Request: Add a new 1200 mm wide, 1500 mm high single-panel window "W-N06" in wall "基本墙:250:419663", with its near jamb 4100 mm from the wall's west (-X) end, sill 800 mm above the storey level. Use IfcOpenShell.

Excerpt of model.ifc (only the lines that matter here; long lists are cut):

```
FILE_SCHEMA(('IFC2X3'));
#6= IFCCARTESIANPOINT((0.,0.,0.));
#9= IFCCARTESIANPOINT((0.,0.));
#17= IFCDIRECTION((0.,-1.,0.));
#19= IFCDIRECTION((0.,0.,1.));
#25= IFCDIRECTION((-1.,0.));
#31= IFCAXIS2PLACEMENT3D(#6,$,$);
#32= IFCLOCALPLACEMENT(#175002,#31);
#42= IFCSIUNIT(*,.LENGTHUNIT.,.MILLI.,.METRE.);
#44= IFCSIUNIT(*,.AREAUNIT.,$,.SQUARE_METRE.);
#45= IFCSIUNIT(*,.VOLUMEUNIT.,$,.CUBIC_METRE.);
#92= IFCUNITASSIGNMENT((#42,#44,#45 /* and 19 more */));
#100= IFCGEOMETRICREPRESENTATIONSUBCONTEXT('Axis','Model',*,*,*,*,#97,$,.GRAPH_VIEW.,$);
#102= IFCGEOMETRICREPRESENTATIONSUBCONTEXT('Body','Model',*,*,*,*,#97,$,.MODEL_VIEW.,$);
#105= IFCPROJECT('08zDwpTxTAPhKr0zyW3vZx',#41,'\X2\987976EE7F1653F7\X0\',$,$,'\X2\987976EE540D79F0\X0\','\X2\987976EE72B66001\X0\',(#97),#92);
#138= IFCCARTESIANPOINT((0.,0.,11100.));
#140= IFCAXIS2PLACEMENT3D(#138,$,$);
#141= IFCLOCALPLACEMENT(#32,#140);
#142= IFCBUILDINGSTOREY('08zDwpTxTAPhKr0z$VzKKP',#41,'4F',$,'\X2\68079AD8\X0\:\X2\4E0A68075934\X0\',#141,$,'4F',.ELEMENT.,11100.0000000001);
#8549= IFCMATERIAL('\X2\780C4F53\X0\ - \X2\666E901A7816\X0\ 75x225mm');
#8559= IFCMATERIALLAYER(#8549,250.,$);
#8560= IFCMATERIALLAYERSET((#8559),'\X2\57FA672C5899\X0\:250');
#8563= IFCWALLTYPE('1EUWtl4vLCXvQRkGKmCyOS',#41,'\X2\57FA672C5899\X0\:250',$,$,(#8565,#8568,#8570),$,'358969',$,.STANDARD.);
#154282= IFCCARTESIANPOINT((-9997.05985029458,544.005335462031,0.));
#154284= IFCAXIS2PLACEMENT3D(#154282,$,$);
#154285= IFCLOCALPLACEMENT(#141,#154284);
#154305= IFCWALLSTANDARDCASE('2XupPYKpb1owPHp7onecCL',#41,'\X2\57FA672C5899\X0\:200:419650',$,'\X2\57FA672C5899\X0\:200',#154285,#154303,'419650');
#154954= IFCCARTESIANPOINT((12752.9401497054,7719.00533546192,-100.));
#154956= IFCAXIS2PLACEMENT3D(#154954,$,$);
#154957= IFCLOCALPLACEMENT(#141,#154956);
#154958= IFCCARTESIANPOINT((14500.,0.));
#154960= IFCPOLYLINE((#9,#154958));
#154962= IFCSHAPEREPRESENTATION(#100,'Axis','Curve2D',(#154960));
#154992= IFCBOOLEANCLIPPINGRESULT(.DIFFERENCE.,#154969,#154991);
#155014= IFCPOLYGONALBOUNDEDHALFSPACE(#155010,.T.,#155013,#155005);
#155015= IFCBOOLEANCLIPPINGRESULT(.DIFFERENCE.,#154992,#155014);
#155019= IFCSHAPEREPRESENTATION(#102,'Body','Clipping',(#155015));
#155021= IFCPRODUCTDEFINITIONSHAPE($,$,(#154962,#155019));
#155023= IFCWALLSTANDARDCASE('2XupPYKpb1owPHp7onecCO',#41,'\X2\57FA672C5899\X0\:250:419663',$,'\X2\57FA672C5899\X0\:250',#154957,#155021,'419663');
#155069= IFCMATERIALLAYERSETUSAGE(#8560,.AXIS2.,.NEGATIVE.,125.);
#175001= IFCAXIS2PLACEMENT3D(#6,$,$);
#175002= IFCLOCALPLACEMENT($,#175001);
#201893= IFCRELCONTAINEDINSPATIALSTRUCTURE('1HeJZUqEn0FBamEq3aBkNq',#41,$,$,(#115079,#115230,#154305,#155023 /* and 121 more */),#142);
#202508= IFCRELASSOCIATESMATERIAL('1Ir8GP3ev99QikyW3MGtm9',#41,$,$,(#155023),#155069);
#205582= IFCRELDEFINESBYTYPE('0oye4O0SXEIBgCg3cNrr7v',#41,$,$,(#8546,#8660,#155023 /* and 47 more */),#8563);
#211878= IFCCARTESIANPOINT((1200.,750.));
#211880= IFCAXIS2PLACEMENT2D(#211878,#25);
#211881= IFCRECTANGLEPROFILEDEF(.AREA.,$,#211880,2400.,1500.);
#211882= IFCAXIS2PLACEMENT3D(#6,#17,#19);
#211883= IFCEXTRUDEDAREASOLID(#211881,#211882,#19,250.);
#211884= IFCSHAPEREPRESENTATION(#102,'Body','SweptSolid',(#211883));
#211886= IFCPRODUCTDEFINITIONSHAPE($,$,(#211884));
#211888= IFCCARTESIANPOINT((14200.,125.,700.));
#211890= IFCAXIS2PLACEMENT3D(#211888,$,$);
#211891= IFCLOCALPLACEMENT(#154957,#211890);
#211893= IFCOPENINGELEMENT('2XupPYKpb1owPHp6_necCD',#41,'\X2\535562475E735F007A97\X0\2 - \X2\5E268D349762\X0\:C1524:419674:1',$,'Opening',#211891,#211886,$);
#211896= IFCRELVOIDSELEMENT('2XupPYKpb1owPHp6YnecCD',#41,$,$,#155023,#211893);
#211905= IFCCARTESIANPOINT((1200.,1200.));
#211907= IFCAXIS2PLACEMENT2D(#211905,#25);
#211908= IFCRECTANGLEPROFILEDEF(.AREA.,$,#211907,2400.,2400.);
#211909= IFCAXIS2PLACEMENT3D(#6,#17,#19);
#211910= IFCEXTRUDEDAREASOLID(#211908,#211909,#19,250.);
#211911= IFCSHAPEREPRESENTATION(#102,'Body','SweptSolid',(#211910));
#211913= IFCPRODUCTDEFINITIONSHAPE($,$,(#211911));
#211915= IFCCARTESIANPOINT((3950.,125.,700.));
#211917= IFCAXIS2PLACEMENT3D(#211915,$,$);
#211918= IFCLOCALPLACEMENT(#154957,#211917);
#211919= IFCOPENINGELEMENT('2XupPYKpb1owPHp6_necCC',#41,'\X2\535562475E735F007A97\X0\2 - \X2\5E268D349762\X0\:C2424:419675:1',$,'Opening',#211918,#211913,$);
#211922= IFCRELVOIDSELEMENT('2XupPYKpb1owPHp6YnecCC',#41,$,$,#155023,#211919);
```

```python
import numpy as np
import ifcopenshell
import ifcopenshell.api.feature
import ifcopenshell.api.geometry
import ifcopenshell.api.root
import ifcopenshell.api.spatial
import ifcopenshell.api.type
import ifcopenshell.geom
import ifcopenshell.util.element
import ifcopenshell.util.placement
import ifcopenshell.util.representation
import ifcopenshell.util.shape
import ifcopenshell.util.unit

model = ifcopenshell.open("model.ifc")
unit_scale = ifcopenshell.util.unit.calculate_unit_scale(model)
settings = ifcopenshell.geom.settings()


def volume(element):
    """Net volume in cubic metres, openings subtracted."""
    shape = ifcopenshell.geom.create_shape(settings, element)
    return ifcopenshell.util.shape.get_volume(shape.geometry)


wall = model.by_guid("2XupPYKpb1owPHp7onecCO")
storey = ifcopenshell.util.element.get_container(wall, ifc_class="IfcBuildingStorey")
context = ifcopenshell.util.representation.get_context(model, "Model", "Body", "MODEL_VIEW")
before = volume(wall)

width, height, from_end, sill = 1.2, 1.5, 4.1, 0.8  # metres

# The wall runs along its own X axis, and the end named is its -X end.
wall_shape = ifcopenshell.geom.create_shape(settings, wall)
x, y, z = ifcopenshell.util.shape.get_vertices(wall_shape.geometry).T
start = x.min() + from_end
face, thickness = float(y.min()), float(y.max() - y.min())
wall_matrix = ifcopenshell.util.placement.get_local_placement(wall.ObjectPlacement)
level = ifcopenshell.util.placement.get_local_placement(storey.ObjectPlacement)[2, 3]


def in_wall(x, y):
    """Placement at x, y metres in the wall's axes, at sill height."""
    matrix = wall_matrix.copy()
    matrix[:, 3] = wall_matrix @ np.array([x / unit_scale, y / unit_scale, 0.0, 1.0])
    matrix[2, 3] = level + sill / unit_scale
    return matrix


# Opening: a box that overshoots both wall faces by 50 mm.
opening = ifcopenshell.api.root.create_entity(model, ifc_class="IfcOpeningElement")
box = ifcopenshell.api.geometry.add_wall_representation(
    model, context=context, length=width, height=height, thickness=thickness + 0.1
)
ifcopenshell.api.geometry.assign_representation(model, product=opening, representation=box)
ifcopenshell.api.geometry.edit_object_placement(model, product=opening, matrix=in_wall(start, face - 0.05), is_si=False)
ifcopenshell.api.feature.add_feature(model, feature=opening, element=wall)

window = ifcopenshell.api.root.create_entity(model, ifc_class="IfcWindow", name="W-N06")
window.OverallWidth, window.OverallHeight = width / unit_scale, height / unit_scale
body = ifcopenshell.api.geometry.add_window_representation(
    model,
    context=context,
    overall_width=window.OverallWidth,
    overall_height=window.OverallHeight,
    partition_type="SINGLE_PANEL",
)
ifcopenshell.api.geometry.assign_representation(model, product=window, representation=body)
ifcopenshell.api.spatial.assign_container(model, products=[window], relating_structure=storey)
fills = ifcopenshell.api.feature.add_filling(model, opening=opening, element=window)
fills.OwnerHistory = window.OwnerHistory  # required in IFC2X3

# IFC2X3 keeps the operation on the window style.
style = ifcopenshell.api.root.create_entity(model, ifc_class="IfcWindowStyle", name="W-N06")
style.OperationType, style.ConstructionType = "SINGLE_PANEL", "NOTDEFINED"
style.ParameterTakesPrecedence = style.Sizeable = False
ifcopenshell.api.type.assign_type(model, related_objects=[window], relating_type=style)

# Centre the window in the wall's thickness.
ifcopenshell.api.geometry.edit_object_placement(model, product=window, matrix=in_wall(start, face), is_si=False)
window_shape = ifcopenshell.geom.create_shape(settings, window)
depth = ifcopenshell.util.shape.get_vertices(window_shape.geometry)[:, 1]
offset = face + thickness / 2 - (depth.min() + depth.max()) / 2
ifcopenshell.api.geometry.edit_object_placement(model, product=window, matrix=in_wall(start, offset), is_si=False)

after = volume(wall)

print(f"wall volume {before:.3f} -> {after:.3f} m3")

model.write("model_rev.ifc")
```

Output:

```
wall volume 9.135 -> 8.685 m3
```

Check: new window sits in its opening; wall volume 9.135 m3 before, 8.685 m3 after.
